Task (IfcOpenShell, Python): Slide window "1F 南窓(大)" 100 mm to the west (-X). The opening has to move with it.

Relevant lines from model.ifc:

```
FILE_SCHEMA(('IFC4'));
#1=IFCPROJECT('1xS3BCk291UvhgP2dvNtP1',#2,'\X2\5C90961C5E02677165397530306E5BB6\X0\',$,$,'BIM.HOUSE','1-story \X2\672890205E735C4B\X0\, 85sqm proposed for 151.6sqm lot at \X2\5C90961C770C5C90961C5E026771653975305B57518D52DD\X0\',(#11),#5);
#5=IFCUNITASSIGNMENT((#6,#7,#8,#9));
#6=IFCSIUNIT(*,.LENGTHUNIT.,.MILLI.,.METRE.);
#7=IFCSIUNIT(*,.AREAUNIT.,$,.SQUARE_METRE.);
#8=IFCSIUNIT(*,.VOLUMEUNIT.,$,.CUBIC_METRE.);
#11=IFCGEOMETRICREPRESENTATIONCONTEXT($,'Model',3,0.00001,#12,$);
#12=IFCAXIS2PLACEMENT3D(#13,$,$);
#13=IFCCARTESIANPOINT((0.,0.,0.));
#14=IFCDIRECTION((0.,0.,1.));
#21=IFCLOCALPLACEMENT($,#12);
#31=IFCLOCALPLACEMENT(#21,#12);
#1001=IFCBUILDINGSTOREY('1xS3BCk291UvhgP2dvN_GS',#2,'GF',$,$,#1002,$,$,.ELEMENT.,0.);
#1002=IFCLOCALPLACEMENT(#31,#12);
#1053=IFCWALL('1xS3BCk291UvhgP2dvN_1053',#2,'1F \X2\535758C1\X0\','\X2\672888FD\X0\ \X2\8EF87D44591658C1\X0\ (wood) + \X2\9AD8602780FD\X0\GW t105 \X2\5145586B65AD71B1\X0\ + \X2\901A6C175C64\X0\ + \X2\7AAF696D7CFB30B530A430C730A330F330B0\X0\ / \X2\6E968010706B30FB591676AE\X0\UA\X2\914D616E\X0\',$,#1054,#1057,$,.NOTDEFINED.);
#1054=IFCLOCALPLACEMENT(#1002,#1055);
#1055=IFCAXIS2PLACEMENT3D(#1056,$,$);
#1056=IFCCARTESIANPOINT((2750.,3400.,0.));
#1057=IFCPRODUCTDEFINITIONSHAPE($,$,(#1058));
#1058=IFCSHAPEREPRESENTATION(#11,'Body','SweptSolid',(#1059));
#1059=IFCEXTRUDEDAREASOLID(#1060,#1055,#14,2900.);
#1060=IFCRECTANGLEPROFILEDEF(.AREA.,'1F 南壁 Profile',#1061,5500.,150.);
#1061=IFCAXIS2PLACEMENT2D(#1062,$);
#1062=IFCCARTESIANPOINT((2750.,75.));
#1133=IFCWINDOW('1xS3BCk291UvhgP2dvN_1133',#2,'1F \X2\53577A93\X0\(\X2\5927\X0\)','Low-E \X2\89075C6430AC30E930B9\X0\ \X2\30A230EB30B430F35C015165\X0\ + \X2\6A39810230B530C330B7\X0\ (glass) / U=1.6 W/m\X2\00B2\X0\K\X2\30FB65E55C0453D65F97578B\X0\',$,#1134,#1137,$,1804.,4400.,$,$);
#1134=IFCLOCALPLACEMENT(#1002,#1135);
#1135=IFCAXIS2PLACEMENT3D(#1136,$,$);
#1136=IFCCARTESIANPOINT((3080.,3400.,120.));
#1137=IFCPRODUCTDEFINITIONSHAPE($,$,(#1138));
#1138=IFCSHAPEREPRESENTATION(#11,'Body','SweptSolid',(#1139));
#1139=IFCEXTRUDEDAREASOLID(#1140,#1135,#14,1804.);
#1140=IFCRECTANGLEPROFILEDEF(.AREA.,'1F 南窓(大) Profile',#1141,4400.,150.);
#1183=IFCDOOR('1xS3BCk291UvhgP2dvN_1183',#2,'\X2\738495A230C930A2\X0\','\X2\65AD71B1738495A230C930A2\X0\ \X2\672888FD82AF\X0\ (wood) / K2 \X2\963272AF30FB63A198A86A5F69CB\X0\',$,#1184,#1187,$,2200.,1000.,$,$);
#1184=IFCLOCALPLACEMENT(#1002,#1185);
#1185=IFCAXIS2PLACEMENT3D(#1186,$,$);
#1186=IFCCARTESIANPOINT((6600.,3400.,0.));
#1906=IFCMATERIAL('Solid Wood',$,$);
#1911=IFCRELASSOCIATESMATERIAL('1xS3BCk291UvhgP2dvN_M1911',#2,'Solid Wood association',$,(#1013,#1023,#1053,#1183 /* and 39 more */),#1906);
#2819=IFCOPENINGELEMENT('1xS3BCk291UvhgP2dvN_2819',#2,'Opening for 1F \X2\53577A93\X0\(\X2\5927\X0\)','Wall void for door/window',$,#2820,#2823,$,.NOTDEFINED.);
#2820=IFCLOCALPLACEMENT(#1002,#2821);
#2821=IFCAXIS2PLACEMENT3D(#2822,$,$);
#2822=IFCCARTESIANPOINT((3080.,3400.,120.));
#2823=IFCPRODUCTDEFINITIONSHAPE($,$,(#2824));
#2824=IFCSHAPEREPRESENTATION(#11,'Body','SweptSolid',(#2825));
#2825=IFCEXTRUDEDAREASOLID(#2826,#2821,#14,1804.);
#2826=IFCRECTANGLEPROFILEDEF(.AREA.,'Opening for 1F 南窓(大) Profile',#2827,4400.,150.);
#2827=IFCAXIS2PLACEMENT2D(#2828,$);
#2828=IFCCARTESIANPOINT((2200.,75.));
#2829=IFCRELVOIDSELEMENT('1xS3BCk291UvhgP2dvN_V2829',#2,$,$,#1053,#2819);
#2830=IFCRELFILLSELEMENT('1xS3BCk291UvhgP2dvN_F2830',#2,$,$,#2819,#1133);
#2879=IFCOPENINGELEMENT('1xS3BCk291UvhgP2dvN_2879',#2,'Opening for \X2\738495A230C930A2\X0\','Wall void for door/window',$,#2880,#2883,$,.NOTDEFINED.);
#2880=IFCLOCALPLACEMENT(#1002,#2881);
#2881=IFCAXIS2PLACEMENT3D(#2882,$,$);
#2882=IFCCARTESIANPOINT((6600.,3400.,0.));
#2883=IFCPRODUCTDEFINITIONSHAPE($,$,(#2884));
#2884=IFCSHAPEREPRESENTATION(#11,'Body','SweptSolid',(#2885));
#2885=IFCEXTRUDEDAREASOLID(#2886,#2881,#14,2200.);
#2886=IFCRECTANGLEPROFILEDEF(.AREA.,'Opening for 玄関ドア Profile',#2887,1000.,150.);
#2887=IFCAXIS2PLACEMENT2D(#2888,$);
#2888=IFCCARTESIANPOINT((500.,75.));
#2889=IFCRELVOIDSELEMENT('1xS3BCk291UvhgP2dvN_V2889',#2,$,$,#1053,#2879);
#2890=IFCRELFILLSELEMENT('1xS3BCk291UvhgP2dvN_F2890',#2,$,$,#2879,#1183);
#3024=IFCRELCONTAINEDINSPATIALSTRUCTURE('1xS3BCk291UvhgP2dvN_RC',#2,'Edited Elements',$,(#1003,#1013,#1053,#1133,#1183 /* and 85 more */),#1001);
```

```python
import ifcopenshell
import ifcopenshell.api.geometry
import ifcopenshell.util.placement
import ifcopenshell.util.unit

model = ifcopenshell.open("model.ifc")
unit_scale = ifcopenshell.util.unit.calculate_unit_scale(model)

window = model.by_guid("1xS3BCk291UvhgP2dvN_1133")
opening = window.FillsVoids[0].RelatingOpeningElement
wall = opening.VoidsElements[0].RelatingBuildingElement

wall_matrix = ifcopenshell.util.placement.get_local_placement(wall.ObjectPlacement)
shift = wall_matrix[:3, 0] * -0.1 / unit_scale
before = ifcopenshell.util.placement.get_local_placement(window.ObjectPlacement)[:3, 3].copy()

# The window is not placed relative to its opening, so move both.
for product in (opening, window):
    matrix = ifcopenshell.util.placement.get_local_placement(product.ObjectPlacement)
    matrix[:3, 3] += shift
    ifcopenshell.api.geometry.edit_object_placement(model, product=product, matrix=matrix, is_si=False)

after = ifcopenshell.util.placement.get_local_placement(window.ObjectPlacement)[:3, 3]
print("window moved by", (after - before).round(3) + 0.0)

model.write("model_updated.ifc")
```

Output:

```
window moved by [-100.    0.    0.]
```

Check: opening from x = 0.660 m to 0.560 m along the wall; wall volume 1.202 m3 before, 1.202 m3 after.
